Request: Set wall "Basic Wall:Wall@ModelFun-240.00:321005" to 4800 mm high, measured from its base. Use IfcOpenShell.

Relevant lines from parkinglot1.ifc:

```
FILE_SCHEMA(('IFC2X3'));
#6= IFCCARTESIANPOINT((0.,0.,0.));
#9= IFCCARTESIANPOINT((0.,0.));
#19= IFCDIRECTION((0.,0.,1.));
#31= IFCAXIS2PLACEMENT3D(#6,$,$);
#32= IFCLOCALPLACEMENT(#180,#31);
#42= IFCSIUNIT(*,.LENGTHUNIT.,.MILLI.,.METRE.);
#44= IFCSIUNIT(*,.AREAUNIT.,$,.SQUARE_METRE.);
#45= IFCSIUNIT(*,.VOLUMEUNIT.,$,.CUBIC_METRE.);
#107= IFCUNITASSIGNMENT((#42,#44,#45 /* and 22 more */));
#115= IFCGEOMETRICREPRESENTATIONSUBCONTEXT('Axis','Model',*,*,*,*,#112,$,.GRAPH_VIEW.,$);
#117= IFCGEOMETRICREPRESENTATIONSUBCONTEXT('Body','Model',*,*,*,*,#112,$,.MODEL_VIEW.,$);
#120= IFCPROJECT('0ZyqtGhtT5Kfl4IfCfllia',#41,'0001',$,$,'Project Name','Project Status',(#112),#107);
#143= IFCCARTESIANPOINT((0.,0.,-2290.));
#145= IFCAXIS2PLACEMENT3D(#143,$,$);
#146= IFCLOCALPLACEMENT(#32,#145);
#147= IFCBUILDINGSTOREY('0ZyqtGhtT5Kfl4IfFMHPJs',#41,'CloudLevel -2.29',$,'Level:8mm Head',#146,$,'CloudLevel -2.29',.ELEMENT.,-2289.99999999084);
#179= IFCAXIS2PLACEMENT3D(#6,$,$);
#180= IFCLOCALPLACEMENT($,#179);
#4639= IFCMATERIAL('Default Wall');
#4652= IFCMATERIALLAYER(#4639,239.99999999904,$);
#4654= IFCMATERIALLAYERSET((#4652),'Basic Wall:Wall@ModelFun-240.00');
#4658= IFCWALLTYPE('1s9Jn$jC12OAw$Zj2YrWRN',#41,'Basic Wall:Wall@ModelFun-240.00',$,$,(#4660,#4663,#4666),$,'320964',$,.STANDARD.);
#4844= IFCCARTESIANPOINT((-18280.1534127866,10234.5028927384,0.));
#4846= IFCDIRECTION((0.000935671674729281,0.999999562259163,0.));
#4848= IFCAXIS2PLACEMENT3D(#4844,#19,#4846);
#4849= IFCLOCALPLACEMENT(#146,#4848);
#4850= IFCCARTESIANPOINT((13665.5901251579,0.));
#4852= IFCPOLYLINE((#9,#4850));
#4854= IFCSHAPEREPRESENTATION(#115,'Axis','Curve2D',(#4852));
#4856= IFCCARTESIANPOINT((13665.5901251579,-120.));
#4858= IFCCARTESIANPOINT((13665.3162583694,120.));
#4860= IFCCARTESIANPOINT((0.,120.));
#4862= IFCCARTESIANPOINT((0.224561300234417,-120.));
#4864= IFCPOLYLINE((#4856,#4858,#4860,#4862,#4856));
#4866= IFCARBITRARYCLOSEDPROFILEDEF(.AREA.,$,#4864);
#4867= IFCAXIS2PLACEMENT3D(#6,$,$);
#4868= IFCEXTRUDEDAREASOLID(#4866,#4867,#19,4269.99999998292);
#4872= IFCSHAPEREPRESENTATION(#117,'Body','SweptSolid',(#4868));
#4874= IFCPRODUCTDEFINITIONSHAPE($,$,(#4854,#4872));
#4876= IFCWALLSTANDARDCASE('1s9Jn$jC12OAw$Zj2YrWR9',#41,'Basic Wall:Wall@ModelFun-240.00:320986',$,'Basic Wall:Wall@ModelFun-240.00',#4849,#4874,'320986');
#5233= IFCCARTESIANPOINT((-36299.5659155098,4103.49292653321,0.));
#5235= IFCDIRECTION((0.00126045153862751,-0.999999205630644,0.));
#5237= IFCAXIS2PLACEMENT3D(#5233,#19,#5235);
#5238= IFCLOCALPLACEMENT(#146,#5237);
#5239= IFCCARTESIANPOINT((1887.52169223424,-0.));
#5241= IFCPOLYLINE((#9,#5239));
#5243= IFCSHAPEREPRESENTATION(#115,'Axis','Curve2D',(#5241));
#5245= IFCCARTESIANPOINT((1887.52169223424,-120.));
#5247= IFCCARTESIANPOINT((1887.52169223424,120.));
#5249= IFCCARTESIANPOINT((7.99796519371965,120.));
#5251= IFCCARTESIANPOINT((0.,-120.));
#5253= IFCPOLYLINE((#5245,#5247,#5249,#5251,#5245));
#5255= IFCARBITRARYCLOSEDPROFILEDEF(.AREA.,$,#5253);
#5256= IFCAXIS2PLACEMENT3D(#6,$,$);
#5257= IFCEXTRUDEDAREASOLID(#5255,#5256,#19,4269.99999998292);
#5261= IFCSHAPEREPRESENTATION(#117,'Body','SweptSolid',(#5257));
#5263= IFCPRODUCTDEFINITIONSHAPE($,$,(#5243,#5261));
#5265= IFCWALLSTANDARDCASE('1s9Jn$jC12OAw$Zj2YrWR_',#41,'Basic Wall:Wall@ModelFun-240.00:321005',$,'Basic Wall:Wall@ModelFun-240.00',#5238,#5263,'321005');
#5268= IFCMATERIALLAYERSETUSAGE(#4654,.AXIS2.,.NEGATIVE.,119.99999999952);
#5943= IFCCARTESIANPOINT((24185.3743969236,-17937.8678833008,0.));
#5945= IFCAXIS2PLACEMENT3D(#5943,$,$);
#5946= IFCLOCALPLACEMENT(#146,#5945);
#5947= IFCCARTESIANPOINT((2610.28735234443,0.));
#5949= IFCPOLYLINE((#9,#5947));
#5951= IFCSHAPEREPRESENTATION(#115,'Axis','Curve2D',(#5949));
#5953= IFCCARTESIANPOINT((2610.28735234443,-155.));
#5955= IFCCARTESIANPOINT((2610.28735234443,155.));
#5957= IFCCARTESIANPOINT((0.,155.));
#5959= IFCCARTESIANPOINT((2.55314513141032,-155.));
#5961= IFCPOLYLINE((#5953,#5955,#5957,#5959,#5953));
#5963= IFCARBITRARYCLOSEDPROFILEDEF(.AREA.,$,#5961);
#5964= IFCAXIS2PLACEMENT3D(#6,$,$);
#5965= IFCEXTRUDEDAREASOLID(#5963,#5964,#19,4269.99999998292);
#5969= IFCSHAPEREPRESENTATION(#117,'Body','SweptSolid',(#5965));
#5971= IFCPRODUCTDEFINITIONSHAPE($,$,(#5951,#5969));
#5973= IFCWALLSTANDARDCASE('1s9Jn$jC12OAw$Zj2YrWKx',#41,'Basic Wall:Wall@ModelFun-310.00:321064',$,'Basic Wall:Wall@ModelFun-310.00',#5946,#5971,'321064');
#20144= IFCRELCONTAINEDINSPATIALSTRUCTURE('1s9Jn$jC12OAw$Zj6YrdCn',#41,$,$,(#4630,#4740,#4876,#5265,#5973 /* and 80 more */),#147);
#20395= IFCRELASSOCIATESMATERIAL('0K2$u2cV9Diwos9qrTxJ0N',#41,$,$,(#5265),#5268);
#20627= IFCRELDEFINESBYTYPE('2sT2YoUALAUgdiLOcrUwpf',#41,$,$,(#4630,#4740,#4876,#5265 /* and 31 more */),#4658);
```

```python
import ifcopenshell
import ifcopenshell.geom
import ifcopenshell.util.representation
import ifcopenshell.util.shape
import ifcopenshell.util.unit

model = ifcopenshell.open("parkinglot1.ifc")
unit_scale = ifcopenshell.util.unit.calculate_unit_scale(model)
settings = ifcopenshell.geom.settings()


def volume(element):
    """Net volume in cubic metres, openings subtracted."""
    shape = ifcopenshell.geom.create_shape(settings, element)
    return ifcopenshell.util.shape.get_volume(shape.geometry)


wall = model.by_id(5265)
before = volume(wall)

body = ifcopenshell.util.representation.get_representation(wall, "Model", "Body")
solid = body.Items[0]
old_height = solid.Depth
solid.Depth = 4.8 / unit_scale
after = volume(wall)

print(f"height {old_height:g} -> {solid.Depth:g}, volume {before:.3f} -> {after:.3f} m3")

model.write("parkinglot1_rev.ifc")
```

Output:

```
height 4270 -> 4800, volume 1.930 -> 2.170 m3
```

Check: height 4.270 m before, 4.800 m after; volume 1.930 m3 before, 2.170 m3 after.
